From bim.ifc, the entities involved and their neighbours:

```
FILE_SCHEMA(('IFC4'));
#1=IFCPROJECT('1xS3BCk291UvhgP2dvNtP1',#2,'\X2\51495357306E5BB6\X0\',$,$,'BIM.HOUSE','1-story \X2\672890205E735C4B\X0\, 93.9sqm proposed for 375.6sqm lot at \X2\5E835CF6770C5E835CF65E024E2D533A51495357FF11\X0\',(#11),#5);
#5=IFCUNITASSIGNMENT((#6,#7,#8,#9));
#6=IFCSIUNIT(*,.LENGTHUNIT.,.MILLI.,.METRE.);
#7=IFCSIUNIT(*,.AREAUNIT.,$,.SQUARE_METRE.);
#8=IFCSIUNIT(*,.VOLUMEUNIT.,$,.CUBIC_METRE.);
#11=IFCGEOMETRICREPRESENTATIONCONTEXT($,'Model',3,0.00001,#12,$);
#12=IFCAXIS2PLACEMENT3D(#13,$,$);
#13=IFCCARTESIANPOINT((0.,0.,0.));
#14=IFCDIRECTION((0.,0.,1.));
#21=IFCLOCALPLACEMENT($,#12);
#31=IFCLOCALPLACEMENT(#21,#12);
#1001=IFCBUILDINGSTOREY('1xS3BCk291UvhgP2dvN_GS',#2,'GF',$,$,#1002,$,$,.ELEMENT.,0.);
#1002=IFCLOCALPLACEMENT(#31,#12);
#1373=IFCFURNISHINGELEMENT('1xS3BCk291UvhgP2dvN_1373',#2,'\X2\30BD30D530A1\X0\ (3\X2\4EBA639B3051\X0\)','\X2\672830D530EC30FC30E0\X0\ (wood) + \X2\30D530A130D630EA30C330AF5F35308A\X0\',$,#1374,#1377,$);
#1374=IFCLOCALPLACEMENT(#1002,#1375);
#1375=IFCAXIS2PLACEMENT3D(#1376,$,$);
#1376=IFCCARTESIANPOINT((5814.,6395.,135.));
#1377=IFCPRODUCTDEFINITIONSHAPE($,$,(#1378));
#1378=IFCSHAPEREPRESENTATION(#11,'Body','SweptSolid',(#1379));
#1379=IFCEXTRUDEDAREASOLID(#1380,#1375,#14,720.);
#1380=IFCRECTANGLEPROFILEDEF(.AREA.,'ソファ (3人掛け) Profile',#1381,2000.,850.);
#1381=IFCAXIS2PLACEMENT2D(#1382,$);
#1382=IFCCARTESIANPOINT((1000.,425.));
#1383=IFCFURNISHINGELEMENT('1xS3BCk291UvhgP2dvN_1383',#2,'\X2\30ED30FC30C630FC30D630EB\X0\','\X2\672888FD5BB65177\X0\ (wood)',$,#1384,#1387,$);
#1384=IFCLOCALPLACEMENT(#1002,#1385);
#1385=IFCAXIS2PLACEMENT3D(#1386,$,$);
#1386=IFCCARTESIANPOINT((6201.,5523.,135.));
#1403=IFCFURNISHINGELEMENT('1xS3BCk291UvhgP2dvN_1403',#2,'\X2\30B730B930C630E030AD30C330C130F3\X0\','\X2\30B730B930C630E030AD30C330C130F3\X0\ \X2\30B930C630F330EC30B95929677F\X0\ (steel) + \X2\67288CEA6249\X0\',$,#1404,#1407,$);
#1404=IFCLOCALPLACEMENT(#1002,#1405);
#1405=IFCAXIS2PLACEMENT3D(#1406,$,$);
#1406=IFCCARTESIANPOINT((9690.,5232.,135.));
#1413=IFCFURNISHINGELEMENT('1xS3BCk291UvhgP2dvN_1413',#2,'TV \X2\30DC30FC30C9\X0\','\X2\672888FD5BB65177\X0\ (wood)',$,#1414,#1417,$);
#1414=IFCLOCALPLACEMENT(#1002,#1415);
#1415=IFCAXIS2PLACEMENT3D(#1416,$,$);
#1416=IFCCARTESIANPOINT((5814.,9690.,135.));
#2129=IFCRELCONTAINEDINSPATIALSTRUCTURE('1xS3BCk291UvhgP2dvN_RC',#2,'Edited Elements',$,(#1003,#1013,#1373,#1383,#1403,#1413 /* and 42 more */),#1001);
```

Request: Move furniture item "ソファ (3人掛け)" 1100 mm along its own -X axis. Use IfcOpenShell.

```python
import ifcopenshell
import ifcopenshell.api.geometry
import ifcopenshell.util.placement

model = ifcopenshell.open("bim.ifc")

item = model.by_guid("1xS3BCk291UvhgP2dvN_1373")
matrix = ifcopenshell.util.placement.get_local_placement(item.ObjectPlacement)
matrix[:3, 3] -= matrix[:3, 0] * 1100.0
ifcopenshell.api.geometry.edit_object_placement(model, product=item, matrix=matrix, is_si=False)

print(ifcopenshell.util.placement.get_local_placement(item.ObjectPlacement).round(3) + 0.0)

model.write("bim-out.ifc")
```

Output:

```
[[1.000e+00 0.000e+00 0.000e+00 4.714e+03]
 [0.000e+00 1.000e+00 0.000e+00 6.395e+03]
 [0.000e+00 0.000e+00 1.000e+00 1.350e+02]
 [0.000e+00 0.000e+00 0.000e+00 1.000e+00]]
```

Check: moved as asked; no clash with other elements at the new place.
